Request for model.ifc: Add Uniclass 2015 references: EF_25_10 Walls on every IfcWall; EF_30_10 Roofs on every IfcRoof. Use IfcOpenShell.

First a look at what the model holds.

```python
import ifcopenshell

model = ifcopenshell.open("model.ifc")
print(model.schema)
print("classifications:", [c.Name for c in model.by_type("IfcClassification")])
for ifc_class in ("IfcDoor", "IfcRoof", "IfcStair", "IfcWall", "IfcWindow"):
    print(ifc_class, len(model.by_type(ifc_class)))
```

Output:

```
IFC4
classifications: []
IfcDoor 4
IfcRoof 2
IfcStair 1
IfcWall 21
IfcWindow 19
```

```python
import ifcopenshell
import ifcopenshell.api.classification

model = ifcopenshell.open("model.ifc")

system = ifcopenshell.api.classification.add_classification(model, classification="Uniclass 2015")

codes = {
    "IfcWall": ("EF_25_10", "Walls"),
    "IfcRoof": ("EF_30_10", "Roofs"),
}
for ifc_class, (code, name) in codes.items():
    products = model.by_type(ifc_class)
    ifcopenshell.api.classification.add_reference(
        model, products=products, classification=system, identification=code, name=name
    )
    print(code, len(products))

model.write("model_updated.ifc")
```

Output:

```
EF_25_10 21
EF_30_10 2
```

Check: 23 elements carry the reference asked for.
